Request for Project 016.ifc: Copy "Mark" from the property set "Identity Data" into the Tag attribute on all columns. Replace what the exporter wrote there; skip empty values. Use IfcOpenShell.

First a look at what the model holds.

```python
import ifcopenshell
import ifcopenshell.util.element

model = ifcopenshell.open("Project 016.ifc")
print(model.schema)
columns = model.by_type("IfcColumn")
print(len(columns), "columns")
for e in columns[:8]:
    source = ifcopenshell.util.element.get_pset(e, "Identity Data", "Mark")
    target = e.Tag
    print(e.id(), repr(source), repr(target), sep=" | ")
```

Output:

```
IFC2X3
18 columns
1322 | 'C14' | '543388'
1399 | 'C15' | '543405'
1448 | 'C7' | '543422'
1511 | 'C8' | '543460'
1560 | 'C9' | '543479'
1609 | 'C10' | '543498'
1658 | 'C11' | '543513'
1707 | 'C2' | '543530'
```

```python
import ifcopenshell
import ifcopenshell.util.element

model = ifcopenshell.open("Project 016.ifc")

count = 0
for e in model.by_type("IfcColumn"):
    value = ifcopenshell.util.element.get_pset(e, "Identity Data", "Mark")
    current = e.Tag
    if not value or not value.strip() or current == value:
        continue
    e.Tag = value
    count += 1

print(count, "columns updated")

model.write("Project 016_rev.ifc")
```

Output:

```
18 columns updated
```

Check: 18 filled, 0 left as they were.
